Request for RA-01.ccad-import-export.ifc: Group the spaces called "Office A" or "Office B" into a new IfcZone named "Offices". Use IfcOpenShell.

First a look at what the model holds.

```python
import ifcopenshell

model = ifcopenshell.open("RA-01.ccad-import-export.ifc")
print(model.schema)
seen = {}
for space in model.by_type("IfcSpace"):
    seen[space.LongName] = seen.get(space.LongName, 0) + 1
for name, count in sorted(seen.items(), key=str):
    print(count, "x", name)
print("zones:", [z.Name for z in model.by_type("IfcZone")][:20])
```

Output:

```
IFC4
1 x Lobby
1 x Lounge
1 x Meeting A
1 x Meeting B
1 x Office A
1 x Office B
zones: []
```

```python
import ifcopenshell
import ifcopenshell.api.group
import ifcopenshell.api.root

model = ifcopenshell.open("RA-01.ccad-import-export.ifc")

names = {"Office A", "Office B"}
spaces = [s for s in model.by_type("IfcSpace") if s.LongName in names]

zone = ifcopenshell.api.root.create_entity(model, ifc_class="IfcZone", name="Offices")
ifcopenshell.api.group.assign_group(model, products=spaces, group=zone)
print(len(spaces), "spaces in", zone.Name)

model.write("RA-01.ccad-import-export_edited.ifc")
```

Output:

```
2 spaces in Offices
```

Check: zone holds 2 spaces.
